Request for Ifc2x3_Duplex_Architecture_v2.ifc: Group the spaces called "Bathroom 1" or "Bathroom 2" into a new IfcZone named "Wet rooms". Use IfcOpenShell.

First a look at what the model holds.

```python
import ifcopenshell

model = ifcopenshell.open("Ifc2x3_Duplex_Architecture_v2.ifc")
print(model.schema)
seen = {}
for space in model.by_type("IfcSpace"):
    seen[space.LongName] = seen.get(space.LongName, 0) + 1
for name, count in sorted(seen.items(), key=str):
    print(count, "x", name)
print("zones:", [z.Name for z in model.by_type("IfcZone")][:20])
```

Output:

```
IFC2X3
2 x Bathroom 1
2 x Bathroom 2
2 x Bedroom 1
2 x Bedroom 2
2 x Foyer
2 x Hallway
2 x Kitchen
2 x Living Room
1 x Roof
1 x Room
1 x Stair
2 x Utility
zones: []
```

```python
import ifcopenshell
import ifcopenshell.api.group
import ifcopenshell.api.root

model = ifcopenshell.open("Ifc2x3_Duplex_Architecture_v2.ifc")

names = {"Bathroom 1", "Bathroom 2"}
spaces = [s for s in model.by_type("IfcSpace") if s.LongName in names]

zone = ifcopenshell.api.root.create_entity(model, ifc_class="IfcZone", name="Wet rooms")
ifcopenshell.api.group.assign_group(model, products=spaces, group=zone)
print(len(spaces), "spaces in", zone.Name)

model.write("Ifc2x3_Duplex_Architecture_v2-out.ifc")
```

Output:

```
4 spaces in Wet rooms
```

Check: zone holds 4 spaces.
